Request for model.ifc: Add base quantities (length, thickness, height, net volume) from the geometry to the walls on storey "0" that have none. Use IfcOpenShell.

First a look at what the model holds.

```python
import ifcopenshell
import ifcopenshell.util.element
import ifcopenshell.util.unit

model = ifcopenshell.open("model.ifc")
print(model.schema)
for unit_type in ("LENGTHUNIT", "AREAUNIT", "VOLUMEUNIT"):
    print(unit_type, ifcopenshell.util.unit.calculate_unit_scale(model, unit_type))
storey = next(s for s in model.by_type("IfcBuildingStorey") if s.Name == "0")
walls = [e for e in ifcopenshell.util.element.get_decomposition(storey) if e.is_a("IfcWall")]
for e in sorted(walls, key=lambda e: e.id()):
    print(e.id(), e.is_a(), e.Name, list(ifcopenshell.util.element.get_psets(e, qtos_only=True)), sep=" | ")
```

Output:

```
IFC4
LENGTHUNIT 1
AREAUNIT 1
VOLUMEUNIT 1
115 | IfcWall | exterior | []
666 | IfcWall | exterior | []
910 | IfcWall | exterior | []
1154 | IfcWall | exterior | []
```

```python
import ifcopenshell
import ifcopenshell.api.pset
import ifcopenshell.geom
import ifcopenshell.util.element
import ifcopenshell.util.shape
import ifcopenshell.util.unit

model = ifcopenshell.open("model.ifc")
unit_scale = ifcopenshell.util.unit.calculate_unit_scale(model)
volume_scale = ifcopenshell.util.unit.calculate_unit_scale(model, "VOLUMEUNIT")
settings = ifcopenshell.geom.settings()

storey = next(s for s in model.by_type("IfcBuildingStorey") if s.Name == "0")
walls = [e for e in ifcopenshell.util.element.get_decomposition(storey) if e.is_a("IfcWall")]

for e in sorted(walls, key=lambda e: e.id()):
    if ifcopenshell.util.element.get_psets(e, qtos_only=True, should_inherit=False):
        continue
    # Geometry comes back in metres, in the element's own axes.
    shape = ifcopenshell.geom.create_shape(settings, e)
    values = {
        "Length": ifcopenshell.util.shape.get_x(shape.geometry) / unit_scale,
        "Width": ifcopenshell.util.shape.get_y(shape.geometry) / unit_scale,
        "Height": ifcopenshell.util.shape.get_z(shape.geometry) / unit_scale,
        "NetVolume": ifcopenshell.util.shape.get_volume(shape.geometry) / volume_scale,
    }
    qto = ifcopenshell.api.pset.add_qto(model, product=e, name="Qto_WallBaseQuantities")
    ifcopenshell.api.pset.edit_qto(model, qto=qto, properties=values)
    print(e.id(), {k: round(v, 3) for k, v in values.items()})

model.write("model_v2.ifc")
```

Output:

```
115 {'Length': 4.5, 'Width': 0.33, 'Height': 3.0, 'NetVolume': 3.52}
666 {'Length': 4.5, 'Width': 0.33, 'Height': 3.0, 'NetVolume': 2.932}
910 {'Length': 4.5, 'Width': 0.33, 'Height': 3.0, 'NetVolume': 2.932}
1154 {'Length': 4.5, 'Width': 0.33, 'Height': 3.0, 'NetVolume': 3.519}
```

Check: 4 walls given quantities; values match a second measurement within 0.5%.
